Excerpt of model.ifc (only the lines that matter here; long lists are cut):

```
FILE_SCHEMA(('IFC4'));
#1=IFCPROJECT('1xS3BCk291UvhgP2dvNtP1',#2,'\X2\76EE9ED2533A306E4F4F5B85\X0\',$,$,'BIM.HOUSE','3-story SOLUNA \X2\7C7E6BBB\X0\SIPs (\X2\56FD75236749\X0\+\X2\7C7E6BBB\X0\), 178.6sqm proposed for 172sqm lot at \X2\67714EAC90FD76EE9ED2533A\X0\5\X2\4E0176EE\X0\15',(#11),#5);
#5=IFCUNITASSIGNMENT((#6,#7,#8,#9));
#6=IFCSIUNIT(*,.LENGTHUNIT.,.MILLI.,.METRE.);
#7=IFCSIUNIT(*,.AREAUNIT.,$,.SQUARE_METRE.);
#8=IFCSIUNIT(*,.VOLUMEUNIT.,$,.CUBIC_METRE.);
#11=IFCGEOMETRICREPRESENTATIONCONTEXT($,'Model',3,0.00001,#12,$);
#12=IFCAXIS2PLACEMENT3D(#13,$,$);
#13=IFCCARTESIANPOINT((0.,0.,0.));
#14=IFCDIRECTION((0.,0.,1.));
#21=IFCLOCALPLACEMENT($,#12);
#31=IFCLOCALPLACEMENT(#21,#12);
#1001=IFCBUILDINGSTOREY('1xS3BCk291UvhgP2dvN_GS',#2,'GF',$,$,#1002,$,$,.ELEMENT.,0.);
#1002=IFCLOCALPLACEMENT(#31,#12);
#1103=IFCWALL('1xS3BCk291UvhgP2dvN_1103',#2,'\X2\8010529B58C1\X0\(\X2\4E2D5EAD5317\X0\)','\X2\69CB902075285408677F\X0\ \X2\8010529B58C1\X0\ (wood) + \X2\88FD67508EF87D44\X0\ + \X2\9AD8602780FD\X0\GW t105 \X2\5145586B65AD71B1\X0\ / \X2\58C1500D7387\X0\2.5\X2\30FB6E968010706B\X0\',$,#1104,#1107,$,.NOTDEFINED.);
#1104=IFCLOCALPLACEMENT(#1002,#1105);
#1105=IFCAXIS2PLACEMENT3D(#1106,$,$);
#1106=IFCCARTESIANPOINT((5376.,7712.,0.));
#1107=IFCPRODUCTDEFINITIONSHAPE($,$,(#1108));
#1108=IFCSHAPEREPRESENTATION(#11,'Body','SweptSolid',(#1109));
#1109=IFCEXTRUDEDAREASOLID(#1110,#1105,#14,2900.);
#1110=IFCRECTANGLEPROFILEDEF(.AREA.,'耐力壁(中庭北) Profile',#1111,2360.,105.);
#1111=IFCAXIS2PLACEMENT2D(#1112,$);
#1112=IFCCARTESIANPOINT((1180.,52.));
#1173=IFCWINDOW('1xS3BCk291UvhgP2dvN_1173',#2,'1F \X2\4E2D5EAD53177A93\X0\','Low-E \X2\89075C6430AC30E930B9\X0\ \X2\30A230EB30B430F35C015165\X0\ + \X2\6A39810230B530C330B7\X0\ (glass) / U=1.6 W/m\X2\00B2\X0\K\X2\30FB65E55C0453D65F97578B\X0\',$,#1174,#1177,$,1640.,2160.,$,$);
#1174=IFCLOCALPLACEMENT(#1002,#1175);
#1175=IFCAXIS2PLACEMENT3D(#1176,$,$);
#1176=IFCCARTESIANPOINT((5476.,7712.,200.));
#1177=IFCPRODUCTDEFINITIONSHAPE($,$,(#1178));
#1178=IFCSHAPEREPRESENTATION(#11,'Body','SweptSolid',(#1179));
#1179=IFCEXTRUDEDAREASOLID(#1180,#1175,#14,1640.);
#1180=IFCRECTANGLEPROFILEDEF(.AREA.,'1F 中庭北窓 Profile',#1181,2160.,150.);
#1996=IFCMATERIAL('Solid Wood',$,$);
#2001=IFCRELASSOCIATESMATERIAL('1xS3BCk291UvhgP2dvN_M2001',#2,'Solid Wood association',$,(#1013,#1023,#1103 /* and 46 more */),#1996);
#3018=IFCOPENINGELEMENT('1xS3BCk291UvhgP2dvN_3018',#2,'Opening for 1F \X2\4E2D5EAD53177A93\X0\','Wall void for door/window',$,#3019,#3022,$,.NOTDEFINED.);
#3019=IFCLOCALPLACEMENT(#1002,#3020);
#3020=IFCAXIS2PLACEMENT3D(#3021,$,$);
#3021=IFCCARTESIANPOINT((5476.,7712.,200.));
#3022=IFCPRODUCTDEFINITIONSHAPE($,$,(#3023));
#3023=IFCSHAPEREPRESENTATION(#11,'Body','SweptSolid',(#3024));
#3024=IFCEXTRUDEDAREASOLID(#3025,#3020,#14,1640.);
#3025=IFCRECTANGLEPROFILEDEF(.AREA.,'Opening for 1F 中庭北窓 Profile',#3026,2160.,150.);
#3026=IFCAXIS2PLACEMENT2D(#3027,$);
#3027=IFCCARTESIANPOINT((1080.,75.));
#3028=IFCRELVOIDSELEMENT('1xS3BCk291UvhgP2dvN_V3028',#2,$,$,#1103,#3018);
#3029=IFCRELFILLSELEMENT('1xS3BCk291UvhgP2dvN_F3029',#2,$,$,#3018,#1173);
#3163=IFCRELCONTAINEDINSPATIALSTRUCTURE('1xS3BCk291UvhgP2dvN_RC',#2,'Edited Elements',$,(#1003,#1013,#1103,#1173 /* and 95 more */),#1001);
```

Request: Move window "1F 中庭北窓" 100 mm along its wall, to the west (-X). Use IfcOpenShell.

```python
import ifcopenshell
import ifcopenshell.api.geometry
import ifcopenshell.util.placement

model = ifcopenshell.open("model.ifc")

window = model.by_guid("1xS3BCk291UvhgP2dvN_1173")
opening = window.FillsVoids[0].RelatingOpeningElement
wall = opening.VoidsElements[0].RelatingBuildingElement

wall_matrix = ifcopenshell.util.placement.get_local_placement(wall.ObjectPlacement)
shift = wall_matrix[:3, 0] * -100.0
before = ifcopenshell.util.placement.get_local_placement(window.ObjectPlacement)[:3, 3].copy()

# The window is not placed relative to its opening, so move both.
for product in (opening, window):
    matrix = ifcopenshell.util.placement.get_local_placement(product.ObjectPlacement)
    matrix[:3, 3] += shift
    ifcopenshell.api.geometry.edit_object_placement(model, product=product, matrix=matrix, is_si=False)

after = ifcopenshell.util.placement.get_local_placement(window.ObjectPlacement)[:3, 3]
print("window moved by", (after - before).round(3) + 0.0)

model.write("model-out.ifc")
```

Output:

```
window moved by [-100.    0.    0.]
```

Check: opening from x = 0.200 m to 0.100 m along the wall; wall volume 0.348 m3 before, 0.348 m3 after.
